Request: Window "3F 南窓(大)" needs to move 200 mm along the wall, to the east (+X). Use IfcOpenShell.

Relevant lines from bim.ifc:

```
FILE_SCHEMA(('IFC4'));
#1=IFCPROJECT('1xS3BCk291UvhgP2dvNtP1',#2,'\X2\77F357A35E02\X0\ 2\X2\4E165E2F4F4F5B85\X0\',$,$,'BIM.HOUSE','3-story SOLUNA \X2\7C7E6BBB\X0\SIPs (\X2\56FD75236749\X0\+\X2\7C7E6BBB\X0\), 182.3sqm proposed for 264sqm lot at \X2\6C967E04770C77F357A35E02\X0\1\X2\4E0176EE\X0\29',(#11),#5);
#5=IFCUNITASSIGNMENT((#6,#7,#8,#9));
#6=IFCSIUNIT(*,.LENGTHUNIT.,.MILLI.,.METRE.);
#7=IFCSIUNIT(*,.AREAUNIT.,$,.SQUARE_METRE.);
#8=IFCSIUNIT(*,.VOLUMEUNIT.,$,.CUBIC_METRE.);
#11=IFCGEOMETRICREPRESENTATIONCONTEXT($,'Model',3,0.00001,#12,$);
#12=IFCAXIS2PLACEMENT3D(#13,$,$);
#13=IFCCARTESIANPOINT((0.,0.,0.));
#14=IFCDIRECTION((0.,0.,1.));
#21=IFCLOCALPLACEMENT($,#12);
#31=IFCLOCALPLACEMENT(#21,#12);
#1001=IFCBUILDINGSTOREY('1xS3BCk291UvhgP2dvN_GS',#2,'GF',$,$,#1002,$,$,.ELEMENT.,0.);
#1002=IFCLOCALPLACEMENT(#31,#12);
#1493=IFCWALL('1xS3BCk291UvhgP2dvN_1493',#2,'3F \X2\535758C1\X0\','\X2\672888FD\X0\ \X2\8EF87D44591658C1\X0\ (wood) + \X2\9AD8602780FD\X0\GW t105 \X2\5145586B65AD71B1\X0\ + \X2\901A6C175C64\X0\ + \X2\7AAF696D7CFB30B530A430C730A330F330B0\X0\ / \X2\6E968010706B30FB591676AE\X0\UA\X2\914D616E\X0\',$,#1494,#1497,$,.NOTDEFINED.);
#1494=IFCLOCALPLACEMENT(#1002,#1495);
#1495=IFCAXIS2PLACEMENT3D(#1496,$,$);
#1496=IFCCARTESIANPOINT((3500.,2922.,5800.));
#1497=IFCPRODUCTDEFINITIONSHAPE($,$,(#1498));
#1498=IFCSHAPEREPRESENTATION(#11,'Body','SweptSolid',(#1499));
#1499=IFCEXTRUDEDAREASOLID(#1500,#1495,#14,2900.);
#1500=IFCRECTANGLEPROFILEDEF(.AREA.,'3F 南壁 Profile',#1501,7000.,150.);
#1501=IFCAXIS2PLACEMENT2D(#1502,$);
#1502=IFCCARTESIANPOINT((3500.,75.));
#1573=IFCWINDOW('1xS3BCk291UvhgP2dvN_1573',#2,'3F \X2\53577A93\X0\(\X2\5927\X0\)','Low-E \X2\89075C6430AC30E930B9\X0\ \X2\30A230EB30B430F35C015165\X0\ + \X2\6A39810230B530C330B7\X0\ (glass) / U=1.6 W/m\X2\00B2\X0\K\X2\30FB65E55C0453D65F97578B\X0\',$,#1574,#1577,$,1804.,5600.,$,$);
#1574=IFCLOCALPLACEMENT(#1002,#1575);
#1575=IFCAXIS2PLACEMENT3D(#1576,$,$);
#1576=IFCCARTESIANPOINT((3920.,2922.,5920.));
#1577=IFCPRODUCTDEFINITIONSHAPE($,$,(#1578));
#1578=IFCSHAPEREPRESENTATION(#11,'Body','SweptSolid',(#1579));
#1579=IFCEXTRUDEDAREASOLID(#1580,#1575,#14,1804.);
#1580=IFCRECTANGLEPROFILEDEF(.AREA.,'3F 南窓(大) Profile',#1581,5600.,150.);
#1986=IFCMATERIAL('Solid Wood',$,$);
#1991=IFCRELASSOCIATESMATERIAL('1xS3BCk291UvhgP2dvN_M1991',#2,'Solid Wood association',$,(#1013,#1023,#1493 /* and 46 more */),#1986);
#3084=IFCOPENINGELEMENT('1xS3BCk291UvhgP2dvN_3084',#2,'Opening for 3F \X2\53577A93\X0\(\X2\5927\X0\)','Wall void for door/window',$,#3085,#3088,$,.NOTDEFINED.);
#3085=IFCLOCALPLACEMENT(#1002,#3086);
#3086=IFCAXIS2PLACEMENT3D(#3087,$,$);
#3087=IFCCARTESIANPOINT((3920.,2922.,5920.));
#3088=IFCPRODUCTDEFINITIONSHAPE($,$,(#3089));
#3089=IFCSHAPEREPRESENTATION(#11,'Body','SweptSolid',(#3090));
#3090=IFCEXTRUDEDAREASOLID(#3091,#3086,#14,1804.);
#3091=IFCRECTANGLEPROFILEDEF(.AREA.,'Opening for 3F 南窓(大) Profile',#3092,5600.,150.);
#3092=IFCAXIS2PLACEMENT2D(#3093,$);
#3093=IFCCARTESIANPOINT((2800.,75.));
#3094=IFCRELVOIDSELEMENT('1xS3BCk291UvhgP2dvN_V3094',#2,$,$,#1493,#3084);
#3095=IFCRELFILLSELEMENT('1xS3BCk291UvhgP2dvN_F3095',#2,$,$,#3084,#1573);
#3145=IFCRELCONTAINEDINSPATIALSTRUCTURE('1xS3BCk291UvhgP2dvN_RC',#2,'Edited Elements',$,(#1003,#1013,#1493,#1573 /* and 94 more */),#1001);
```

```python
import ifcopenshell
import ifcopenshell.api.geometry
import ifcopenshell.util.placement
import ifcopenshell.util.unit

model = ifcopenshell.open("bim.ifc")
unit_scale = ifcopenshell.util.unit.calculate_unit_scale(model)

window = model.by_guid("1xS3BCk291UvhgP2dvN_1573")
opening = window.FillsVoids[0].RelatingOpeningElement
wall = opening.VoidsElements[0].RelatingBuildingElement

wall_matrix = ifcopenshell.util.placement.get_local_placement(wall.ObjectPlacement)
shift = wall_matrix[:3, 0] * 0.2 / unit_scale
before = ifcopenshell.util.placement.get_local_placement(window.ObjectPlacement)[:3, 3].copy()

# The window is not placed relative to its opening, so move both.
for product in (opening, window):
    matrix = ifcopenshell.util.placement.get_local_placement(product.ObjectPlacement)
    matrix[:3, 3] += shift
    ifcopenshell.api.geometry.edit_object_placement(model, product=product, matrix=matrix, is_si=False)

after = ifcopenshell.util.placement.get_local_placement(window.ObjectPlacement)[:3, 3]
print("window moved by", (after - before).round(3) + 0.0)

model.write("bim_updated.ifc")
```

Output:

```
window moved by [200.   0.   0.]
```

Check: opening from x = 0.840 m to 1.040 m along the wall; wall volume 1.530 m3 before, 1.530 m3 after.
